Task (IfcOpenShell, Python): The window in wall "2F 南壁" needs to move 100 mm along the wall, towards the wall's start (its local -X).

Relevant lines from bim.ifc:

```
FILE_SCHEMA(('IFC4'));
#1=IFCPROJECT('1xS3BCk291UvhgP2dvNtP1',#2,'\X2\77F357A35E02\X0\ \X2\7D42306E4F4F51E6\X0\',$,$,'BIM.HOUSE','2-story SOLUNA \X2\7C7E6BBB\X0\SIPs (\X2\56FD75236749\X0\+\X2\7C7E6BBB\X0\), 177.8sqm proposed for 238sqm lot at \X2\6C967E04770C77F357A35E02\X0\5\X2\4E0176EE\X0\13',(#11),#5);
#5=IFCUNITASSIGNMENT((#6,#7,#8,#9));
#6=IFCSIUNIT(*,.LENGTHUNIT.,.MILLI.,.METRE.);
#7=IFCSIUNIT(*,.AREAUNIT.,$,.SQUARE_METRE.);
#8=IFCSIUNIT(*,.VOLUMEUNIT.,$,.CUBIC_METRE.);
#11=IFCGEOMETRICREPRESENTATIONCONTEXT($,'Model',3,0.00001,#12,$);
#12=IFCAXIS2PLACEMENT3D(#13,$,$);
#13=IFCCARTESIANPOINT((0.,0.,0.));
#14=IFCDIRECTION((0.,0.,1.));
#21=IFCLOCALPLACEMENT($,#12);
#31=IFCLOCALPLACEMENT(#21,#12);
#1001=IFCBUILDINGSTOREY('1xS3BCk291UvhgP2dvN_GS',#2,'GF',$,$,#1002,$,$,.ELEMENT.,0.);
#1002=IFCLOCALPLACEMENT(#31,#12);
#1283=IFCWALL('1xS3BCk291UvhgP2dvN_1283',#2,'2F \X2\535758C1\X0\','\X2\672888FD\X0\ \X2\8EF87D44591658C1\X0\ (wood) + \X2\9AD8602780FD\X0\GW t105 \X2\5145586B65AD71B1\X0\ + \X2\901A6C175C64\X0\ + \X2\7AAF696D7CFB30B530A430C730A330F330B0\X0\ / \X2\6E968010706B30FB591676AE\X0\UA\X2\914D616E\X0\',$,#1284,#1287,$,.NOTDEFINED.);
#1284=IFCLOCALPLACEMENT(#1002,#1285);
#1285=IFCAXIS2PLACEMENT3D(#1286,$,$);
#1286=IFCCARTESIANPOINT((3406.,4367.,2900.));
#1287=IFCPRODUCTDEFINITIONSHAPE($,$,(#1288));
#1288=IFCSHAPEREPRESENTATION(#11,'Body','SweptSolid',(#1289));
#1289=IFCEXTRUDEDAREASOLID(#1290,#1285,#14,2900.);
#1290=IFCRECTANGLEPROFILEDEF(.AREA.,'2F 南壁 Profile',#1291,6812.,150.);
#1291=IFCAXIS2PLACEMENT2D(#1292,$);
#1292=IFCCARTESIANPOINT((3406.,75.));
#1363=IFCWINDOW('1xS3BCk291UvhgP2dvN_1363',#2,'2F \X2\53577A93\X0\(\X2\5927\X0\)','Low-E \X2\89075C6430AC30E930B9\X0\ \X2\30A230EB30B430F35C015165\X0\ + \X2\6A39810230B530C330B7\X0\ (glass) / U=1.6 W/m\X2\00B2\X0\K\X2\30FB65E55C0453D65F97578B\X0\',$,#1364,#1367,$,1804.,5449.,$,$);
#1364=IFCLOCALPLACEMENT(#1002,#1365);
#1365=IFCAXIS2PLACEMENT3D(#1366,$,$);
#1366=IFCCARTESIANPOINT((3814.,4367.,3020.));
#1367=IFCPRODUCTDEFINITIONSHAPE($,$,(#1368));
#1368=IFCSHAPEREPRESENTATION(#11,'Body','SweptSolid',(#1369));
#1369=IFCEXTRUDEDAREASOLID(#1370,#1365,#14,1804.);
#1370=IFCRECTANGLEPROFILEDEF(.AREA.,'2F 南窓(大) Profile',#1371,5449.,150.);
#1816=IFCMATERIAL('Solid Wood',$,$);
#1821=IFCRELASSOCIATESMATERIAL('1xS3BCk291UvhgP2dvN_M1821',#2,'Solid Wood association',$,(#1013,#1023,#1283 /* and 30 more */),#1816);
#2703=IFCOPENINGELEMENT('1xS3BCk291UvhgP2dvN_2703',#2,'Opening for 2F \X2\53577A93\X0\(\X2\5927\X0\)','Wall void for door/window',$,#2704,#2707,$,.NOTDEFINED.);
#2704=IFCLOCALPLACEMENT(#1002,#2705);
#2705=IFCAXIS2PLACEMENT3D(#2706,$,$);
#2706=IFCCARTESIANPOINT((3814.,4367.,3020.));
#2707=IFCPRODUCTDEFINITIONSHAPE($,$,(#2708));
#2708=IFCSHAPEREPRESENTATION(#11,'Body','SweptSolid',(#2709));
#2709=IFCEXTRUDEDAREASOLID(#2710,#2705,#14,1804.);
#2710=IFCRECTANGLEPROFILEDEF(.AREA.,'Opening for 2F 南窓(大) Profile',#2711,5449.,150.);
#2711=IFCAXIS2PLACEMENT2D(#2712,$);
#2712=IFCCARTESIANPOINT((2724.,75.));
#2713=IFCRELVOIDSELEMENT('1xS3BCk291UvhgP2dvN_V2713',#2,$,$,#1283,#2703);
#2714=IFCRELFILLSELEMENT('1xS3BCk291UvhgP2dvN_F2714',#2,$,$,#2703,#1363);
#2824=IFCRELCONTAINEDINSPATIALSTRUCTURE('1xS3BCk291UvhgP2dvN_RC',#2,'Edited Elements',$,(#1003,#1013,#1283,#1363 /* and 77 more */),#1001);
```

```python
import ifcopenshell
import ifcopenshell.api.geometry
import ifcopenshell.util.placement

model = ifcopenshell.open("bim.ifc")

window = model.by_guid("1xS3BCk291UvhgP2dvN_1363")
opening = window.FillsVoids[0].RelatingOpeningElement
wall = opening.VoidsElements[0].RelatingBuildingElement

wall_matrix = ifcopenshell.util.placement.get_local_placement(wall.ObjectPlacement)
shift = wall_matrix[:3, 0] * -100.0
before = ifcopenshell.util.placement.get_local_placement(window.ObjectPlacement)[:3, 3].copy()

# The window is not placed relative to its opening, so move both.
for product in (opening, window):
    matrix = ifcopenshell.util.placement.get_local_placement(product.ObjectPlacement)
    matrix[:3, 3] += shift
    ifcopenshell.api.geometry.edit_object_placement(model, product=product, matrix=matrix, is_si=False)

after = ifcopenshell.util.placement.get_local_placement(window.ObjectPlacement)[:3, 3]
print("window moved by", (after - before).round(3) + 0.0)

model.write("bim_updated.ifc")
```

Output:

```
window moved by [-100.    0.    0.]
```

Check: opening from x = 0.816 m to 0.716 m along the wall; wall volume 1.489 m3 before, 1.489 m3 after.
